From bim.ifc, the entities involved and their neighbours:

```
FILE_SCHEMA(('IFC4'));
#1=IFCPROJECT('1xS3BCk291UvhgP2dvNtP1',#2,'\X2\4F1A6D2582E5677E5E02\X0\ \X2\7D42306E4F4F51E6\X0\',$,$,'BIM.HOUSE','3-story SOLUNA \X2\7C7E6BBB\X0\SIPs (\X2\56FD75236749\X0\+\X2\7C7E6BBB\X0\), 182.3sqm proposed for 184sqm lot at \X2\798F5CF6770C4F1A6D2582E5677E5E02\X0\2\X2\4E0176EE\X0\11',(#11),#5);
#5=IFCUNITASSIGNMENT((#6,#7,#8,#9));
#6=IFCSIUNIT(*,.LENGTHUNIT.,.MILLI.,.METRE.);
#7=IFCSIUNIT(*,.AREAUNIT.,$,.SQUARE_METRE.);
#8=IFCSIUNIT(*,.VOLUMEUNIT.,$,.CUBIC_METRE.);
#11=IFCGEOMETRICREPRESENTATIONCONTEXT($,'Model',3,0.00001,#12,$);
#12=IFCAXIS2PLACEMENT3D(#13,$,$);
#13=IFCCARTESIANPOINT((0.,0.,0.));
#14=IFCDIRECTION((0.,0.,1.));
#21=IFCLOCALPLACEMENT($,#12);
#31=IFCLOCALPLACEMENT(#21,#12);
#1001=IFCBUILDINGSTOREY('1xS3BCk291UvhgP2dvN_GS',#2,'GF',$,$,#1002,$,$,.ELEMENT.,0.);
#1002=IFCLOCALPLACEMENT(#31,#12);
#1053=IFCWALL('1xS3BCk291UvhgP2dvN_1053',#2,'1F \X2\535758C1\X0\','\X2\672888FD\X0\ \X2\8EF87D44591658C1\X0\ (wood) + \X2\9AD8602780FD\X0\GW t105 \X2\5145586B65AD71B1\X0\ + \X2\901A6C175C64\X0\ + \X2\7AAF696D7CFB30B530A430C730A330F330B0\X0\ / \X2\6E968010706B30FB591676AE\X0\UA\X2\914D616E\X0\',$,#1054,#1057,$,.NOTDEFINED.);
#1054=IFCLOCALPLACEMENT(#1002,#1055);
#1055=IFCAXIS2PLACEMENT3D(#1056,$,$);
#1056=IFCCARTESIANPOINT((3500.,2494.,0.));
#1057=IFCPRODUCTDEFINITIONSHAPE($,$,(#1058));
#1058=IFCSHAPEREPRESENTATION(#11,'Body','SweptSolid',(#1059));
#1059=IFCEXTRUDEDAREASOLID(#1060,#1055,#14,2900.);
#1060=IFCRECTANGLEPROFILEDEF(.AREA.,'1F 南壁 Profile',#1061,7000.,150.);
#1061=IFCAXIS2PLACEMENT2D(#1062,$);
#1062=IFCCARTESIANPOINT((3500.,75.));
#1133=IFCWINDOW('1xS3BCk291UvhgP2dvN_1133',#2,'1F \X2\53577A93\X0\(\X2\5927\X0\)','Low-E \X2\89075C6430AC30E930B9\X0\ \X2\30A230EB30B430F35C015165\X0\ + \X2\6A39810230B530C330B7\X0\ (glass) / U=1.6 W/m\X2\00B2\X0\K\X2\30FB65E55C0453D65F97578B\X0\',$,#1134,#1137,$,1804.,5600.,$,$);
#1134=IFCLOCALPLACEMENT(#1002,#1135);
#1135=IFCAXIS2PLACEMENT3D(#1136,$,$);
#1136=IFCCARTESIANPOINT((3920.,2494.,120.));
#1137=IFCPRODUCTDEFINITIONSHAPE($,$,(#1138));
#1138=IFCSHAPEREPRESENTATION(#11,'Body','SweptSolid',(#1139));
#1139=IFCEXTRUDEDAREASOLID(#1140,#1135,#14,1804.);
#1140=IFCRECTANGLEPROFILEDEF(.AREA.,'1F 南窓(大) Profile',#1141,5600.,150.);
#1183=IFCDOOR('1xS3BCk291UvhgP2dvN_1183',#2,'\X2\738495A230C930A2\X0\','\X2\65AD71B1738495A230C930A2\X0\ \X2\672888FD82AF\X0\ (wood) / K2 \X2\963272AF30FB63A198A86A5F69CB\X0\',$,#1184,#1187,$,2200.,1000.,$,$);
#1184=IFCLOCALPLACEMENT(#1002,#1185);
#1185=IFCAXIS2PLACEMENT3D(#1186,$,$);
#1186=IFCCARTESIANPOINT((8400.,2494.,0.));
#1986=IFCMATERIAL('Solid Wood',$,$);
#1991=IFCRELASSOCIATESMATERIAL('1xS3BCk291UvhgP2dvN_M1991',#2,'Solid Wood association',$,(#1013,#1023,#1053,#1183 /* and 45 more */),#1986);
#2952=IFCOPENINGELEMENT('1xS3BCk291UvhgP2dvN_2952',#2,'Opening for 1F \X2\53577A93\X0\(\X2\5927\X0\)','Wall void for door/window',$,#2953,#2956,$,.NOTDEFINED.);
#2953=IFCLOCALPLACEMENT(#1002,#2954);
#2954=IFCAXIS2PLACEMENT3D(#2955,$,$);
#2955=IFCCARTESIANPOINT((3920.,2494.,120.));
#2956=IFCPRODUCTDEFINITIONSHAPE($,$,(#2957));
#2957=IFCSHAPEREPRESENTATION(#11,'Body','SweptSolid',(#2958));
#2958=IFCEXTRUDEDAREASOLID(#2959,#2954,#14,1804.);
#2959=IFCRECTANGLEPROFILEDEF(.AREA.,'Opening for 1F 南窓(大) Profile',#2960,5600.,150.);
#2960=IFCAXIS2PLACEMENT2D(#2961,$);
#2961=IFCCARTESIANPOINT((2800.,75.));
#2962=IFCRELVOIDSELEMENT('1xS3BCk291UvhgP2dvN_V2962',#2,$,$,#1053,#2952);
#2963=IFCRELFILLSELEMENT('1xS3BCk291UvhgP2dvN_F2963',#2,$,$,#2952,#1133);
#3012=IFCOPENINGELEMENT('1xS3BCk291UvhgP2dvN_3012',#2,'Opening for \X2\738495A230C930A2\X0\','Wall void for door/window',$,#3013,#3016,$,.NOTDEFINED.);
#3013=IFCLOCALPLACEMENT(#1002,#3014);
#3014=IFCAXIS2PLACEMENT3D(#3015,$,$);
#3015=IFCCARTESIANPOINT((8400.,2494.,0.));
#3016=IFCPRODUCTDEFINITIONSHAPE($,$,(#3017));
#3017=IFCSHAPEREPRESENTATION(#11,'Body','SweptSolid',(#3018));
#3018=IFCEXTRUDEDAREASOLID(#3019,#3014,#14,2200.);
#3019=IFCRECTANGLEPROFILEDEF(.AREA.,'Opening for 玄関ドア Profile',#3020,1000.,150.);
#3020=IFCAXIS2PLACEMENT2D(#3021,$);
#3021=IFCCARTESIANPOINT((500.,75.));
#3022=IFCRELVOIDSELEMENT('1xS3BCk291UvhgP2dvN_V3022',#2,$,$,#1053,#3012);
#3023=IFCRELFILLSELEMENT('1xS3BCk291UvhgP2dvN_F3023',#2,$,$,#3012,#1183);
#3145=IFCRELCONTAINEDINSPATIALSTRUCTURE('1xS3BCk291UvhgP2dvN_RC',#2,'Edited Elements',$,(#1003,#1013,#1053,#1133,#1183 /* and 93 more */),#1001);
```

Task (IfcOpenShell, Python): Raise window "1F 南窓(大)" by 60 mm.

```python
import numpy as np
import ifcopenshell
import ifcopenshell.api.geometry
import ifcopenshell.util.placement
import ifcopenshell.util.unit

model = ifcopenshell.open("bim.ifc")
unit_scale = ifcopenshell.util.unit.calculate_unit_scale(model)

window = model.by_id(1133)
opening = window.FillsVoids[0].RelatingOpeningElement
dz = 60.0

shift = np.array([0.0, 0.0, dz])
# The window is not placed relative to its opening, so move both.
for product in (opening, window):
    matrix = ifcopenshell.util.placement.get_local_placement(product.ObjectPlacement)
    matrix[:3, 3] += shift
    ifcopenshell.api.geometry.edit_object_placement(model, product=product, matrix=matrix, is_si=False)

print(f"moved by {dz * unit_scale:+.3f} m")

model.write("bim_edited.ifc")
```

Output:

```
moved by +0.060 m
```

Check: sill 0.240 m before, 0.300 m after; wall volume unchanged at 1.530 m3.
